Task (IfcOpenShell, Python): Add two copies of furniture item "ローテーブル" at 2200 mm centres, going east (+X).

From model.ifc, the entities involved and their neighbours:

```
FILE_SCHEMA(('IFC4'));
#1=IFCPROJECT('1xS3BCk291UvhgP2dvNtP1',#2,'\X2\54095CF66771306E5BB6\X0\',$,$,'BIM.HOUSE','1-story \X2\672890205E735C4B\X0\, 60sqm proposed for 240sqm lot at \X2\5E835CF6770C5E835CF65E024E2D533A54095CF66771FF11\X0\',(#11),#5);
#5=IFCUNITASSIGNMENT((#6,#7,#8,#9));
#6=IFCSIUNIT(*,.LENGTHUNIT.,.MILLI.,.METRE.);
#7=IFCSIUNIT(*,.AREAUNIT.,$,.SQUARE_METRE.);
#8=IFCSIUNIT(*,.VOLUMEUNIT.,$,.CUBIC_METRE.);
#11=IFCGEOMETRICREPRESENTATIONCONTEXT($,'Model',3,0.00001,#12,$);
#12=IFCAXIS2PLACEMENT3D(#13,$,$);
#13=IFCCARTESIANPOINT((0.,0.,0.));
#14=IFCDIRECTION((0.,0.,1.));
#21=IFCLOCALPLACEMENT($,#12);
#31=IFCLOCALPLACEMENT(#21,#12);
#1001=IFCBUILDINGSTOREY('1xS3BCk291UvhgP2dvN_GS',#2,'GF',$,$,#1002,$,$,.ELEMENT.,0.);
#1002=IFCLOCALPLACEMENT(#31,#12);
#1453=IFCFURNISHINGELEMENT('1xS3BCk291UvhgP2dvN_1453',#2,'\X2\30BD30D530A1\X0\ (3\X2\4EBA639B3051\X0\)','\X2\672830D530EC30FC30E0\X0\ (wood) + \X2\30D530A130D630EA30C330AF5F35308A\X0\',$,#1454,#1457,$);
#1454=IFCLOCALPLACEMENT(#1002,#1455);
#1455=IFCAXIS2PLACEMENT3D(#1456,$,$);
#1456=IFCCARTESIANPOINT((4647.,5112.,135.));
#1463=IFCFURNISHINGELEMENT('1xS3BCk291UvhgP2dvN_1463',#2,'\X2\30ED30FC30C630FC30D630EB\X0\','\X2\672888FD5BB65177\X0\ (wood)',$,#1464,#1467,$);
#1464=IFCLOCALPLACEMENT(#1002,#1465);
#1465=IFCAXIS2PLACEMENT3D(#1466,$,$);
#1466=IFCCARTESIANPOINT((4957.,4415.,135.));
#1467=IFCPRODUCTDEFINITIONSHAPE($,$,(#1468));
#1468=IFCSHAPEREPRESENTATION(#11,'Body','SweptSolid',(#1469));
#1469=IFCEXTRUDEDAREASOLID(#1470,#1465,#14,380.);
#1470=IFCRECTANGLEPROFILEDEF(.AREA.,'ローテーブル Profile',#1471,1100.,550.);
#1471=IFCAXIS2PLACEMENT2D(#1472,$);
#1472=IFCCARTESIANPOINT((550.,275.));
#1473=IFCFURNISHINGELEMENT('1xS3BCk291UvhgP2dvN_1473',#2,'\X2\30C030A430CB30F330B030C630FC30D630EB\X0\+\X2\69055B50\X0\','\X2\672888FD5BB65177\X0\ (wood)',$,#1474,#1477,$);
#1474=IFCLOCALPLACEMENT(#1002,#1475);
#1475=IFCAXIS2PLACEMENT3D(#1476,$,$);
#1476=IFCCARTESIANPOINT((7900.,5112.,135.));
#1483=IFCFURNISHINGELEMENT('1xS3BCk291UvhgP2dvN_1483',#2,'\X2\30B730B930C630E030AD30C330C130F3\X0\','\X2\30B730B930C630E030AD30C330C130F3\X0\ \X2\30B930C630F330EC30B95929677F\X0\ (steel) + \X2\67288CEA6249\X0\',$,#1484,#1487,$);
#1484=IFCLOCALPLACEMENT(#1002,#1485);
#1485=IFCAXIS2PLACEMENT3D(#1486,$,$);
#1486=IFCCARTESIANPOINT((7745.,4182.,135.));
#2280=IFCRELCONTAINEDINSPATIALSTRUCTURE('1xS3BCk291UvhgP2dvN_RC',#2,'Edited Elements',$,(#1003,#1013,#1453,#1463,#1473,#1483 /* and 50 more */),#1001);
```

```python
import numpy as np
import ifcopenshell
import ifcopenshell.api.geometry
import ifcopenshell.api.root
import ifcopenshell.util.element
import ifcopenshell.util.placement

model = ifcopenshell.open("model.ifc")


def reuse_history(source, copy):
    """copy_class also copies each property set's owner history, people and application; keep the originals."""
    for rel in copy.IsDefinedBy:
        if rel.is_a("IfcRelDefinesByProperties") and (history := rel.RelatingPropertyDefinition.OwnerHistory):
            rel.RelatingPropertyDefinition.OwnerHistory = source.OwnerHistory
            ifcopenshell.util.element.remove_deep2(model, history)


source = model.by_guid("1xS3BCk291UvhgP2dvN_1463")
base = ifcopenshell.util.placement.get_local_placement(source.ObjectPlacement)
step = np.array([1.0, 0.0, 0.0]) * 2200.0

for i in range(1, 3):
    copy = ifcopenshell.api.root.copy_class(model, product=source)
    copy.Representation = ifcopenshell.util.element.copy_deep(
        model, source.Representation, exclude=["IfcGeometricRepresentationContext", "IfcRepresentationMap"]
    )
    reuse_history(source, copy)
    matrix = base.copy()
    matrix[:3, 3] += i * step
    print("added at", matrix[:3, 3].round(3) + 0.0)
    ifcopenshell.api.geometry.edit_object_placement(model, product=copy, matrix=matrix, is_si=False)

model.write("model-out.ifc")
```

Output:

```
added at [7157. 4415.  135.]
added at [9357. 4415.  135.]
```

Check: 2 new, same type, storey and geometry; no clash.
